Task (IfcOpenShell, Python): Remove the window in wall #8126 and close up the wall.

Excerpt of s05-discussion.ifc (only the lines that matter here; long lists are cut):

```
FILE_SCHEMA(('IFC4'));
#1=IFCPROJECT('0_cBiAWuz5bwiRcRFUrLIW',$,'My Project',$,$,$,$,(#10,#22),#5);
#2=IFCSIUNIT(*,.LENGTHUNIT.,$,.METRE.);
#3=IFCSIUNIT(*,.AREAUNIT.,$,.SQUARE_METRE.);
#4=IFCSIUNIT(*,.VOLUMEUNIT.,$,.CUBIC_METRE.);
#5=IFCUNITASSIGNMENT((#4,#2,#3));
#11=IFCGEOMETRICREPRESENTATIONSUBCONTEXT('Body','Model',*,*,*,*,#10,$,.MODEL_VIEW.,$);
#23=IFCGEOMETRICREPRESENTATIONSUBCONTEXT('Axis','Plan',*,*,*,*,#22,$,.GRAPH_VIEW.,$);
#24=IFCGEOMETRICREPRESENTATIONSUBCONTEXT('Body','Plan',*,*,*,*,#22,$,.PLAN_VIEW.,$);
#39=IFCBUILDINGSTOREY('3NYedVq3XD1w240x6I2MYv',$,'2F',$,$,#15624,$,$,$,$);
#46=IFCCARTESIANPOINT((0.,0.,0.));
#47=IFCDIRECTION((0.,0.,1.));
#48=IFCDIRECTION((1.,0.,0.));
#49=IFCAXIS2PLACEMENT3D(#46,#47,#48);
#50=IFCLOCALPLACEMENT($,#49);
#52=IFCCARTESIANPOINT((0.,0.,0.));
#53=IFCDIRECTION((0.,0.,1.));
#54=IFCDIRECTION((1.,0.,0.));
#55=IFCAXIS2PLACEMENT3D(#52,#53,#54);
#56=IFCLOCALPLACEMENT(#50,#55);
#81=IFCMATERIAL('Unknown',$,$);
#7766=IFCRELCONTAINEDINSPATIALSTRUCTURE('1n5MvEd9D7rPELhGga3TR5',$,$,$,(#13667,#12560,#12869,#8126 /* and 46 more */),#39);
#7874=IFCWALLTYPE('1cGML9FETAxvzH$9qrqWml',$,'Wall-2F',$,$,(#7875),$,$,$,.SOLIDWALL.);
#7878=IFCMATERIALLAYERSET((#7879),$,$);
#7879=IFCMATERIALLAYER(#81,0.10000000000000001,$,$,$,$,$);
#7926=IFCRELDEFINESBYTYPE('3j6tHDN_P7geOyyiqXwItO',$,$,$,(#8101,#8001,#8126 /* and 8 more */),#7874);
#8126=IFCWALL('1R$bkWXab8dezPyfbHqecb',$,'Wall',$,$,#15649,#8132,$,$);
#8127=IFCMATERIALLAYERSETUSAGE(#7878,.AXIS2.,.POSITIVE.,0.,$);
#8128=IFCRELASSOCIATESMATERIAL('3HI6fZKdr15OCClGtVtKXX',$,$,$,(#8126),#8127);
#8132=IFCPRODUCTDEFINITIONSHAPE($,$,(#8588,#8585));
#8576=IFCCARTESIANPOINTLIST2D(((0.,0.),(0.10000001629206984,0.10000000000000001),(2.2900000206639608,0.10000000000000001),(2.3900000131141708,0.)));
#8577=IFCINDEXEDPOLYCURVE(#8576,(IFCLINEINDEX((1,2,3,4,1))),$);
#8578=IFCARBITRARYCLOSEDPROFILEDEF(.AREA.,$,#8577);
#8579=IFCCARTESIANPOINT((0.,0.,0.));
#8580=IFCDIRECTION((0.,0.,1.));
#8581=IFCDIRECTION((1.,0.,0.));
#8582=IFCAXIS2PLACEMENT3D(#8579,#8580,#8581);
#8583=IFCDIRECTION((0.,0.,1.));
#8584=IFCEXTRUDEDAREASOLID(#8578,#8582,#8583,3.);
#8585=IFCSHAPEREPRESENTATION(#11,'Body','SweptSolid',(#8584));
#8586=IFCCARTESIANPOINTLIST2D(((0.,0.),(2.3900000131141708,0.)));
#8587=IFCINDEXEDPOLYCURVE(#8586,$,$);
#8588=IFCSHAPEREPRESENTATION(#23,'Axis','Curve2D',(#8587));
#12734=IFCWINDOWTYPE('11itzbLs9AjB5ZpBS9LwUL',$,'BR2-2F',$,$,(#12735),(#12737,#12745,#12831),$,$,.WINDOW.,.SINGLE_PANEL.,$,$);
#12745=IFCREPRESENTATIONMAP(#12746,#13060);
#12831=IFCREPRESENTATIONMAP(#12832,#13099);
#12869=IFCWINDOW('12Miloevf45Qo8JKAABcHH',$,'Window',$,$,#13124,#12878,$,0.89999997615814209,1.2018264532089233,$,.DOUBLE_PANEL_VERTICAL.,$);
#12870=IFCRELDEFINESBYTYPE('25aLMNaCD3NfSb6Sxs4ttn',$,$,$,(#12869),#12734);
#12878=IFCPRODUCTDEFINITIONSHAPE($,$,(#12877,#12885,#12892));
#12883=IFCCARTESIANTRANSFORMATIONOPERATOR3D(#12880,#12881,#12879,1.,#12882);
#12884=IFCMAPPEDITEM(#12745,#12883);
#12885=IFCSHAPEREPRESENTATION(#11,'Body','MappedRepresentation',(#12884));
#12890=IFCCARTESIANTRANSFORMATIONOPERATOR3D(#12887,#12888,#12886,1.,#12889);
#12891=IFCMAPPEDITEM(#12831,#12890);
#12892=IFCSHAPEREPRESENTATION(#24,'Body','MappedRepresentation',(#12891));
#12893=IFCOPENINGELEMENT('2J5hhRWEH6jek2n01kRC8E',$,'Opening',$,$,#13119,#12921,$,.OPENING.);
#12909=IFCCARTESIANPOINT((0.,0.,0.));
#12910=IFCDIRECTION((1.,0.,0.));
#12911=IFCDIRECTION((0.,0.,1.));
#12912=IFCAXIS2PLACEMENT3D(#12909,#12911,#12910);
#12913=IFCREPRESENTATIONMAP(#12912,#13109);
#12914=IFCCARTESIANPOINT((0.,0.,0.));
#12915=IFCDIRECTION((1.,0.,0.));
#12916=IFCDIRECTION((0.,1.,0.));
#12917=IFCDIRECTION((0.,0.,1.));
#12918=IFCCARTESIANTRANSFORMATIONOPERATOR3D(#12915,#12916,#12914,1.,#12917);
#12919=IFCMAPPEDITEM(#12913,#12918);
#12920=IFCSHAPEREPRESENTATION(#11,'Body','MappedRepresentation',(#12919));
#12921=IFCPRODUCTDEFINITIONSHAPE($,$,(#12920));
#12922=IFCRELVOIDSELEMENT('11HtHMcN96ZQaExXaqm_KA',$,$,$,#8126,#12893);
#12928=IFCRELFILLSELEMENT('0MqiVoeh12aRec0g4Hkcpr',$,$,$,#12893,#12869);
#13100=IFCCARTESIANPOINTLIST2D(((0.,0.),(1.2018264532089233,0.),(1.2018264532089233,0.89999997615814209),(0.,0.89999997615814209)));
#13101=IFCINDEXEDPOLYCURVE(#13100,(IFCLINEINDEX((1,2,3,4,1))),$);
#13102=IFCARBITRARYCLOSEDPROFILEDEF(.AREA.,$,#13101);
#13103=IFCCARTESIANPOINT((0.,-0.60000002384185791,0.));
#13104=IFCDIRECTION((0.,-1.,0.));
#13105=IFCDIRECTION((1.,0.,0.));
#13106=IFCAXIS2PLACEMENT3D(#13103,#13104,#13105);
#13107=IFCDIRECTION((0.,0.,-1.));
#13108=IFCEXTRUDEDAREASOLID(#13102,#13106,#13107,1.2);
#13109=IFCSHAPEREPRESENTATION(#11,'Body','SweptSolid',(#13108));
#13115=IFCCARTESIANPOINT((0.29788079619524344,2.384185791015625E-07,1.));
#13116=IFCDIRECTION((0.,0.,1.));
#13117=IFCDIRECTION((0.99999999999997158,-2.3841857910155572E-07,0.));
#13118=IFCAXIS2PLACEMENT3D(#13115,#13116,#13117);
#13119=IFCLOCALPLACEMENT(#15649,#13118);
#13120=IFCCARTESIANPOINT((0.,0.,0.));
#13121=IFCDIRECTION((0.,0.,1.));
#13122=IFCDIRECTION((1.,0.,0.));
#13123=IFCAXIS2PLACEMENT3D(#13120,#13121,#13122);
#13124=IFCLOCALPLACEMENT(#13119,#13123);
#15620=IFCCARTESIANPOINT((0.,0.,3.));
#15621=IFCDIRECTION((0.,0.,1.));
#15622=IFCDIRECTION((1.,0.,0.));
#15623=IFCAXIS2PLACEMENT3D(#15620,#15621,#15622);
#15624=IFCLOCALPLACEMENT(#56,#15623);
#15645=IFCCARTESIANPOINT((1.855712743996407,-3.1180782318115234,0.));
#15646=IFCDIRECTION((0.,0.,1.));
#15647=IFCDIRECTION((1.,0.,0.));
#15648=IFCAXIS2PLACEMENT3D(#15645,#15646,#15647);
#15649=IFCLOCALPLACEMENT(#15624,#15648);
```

```python
import ifcopenshell
import ifcopenshell.api.feature
import ifcopenshell.api.root
import ifcopenshell.geom
import ifcopenshell.util.shape

model = ifcopenshell.open("s05-discussion.ifc")
settings = ifcopenshell.geom.settings()


def volume(element):
    """Net volume in cubic metres, openings subtracted."""
    shape = ifcopenshell.geom.create_shape(settings, element)
    return ifcopenshell.util.shape.get_volume(shape.geometry)


window = model.by_id(12869)
opening = window.FillsVoids[0].RelatingOpeningElement
wall = opening.VoidsElements[0].RelatingBuildingElement
before = volume(wall)

ifcopenshell.api.root.remove_product(model, product=window)
ifcopenshell.api.feature.remove_feature(model, feature=opening)

after = volume(wall)

print(f"wall volume {before:.3f} -> {after:.3f} m3")

model.write("s05-discussion_updated.ifc")
```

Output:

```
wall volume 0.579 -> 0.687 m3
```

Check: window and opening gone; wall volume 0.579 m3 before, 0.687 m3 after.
